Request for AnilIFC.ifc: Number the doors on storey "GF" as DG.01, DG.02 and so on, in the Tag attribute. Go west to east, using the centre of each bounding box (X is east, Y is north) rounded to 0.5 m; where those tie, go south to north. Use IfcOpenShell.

First a look at what the model holds.

```python
import ifcopenshell
import ifcopenshell.util.element
import ifcopenshell.util.placement

model = ifcopenshell.open("AnilIFC.ifc")
print(model.schema)
storey = next(s for s in model.by_type("IfcBuildingStorey") if s.Name == "GF")
doors = [e for e in ifcopenshell.util.element.get_decomposition(storey) if e.is_a("IfcDoor")]
for e in sorted(doors, key=lambda e: e.id()):
    origin = ifcopenshell.util.placement.get_local_placement(e.ObjectPlacement)[:3, 3]
    print(e.id(), e.Tag, e.Name, origin.round(2) + 0.0, sep=" | ")
```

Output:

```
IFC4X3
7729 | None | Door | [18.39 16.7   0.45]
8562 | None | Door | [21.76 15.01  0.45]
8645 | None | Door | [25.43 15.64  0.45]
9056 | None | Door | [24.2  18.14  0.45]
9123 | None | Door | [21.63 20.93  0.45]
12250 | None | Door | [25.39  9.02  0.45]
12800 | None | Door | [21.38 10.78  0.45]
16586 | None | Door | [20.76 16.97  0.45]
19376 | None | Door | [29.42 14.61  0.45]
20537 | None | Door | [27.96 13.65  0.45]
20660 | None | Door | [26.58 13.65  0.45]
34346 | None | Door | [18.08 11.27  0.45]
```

```python
import ifcopenshell
import ifcopenshell.geom
import ifcopenshell.util.element
import ifcopenshell.util.shape

model = ifcopenshell.open("AnilIFC.ifc")
settings = ifcopenshell.geom.settings()
settings.set("use-world-coords", True)


def centre(element):
    shape = ifcopenshell.geom.create_shape(settings, element)
    return ifcopenshell.util.shape.get_bbox_centroid(shape.geometry)


storey = next(s for s in model.by_type("IfcBuildingStorey") if s.Name == "GF")
doors = [e for e in ifcopenshell.util.element.get_decomposition(storey) if e.is_a("IfcDoor")]

# Insertion points can sit at a corner or the storey origin, so sort by the geometry (in metres).
centres = {e: centre(e) for e in doors}
doors.sort(key=lambda e: (round(centres[e][0] / 0.5), centres[e][1]))

for i, e in enumerate(doors, start=1):
    number = f"DG.{i:02d}"
    e.Tag = number
    print(e.id(), number)

model.write("AnilIFC_v2.ifc")
```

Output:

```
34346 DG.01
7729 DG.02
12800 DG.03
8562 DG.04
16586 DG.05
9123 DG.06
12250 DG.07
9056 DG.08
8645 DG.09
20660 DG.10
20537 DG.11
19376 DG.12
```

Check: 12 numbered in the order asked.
